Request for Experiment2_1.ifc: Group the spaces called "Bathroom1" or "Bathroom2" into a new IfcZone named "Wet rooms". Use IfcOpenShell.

First a look at what the model holds.

```python
import ifcopenshell

model = ifcopenshell.open("Experiment2_1.ifc")
print(model.schema)
seen = {}
for space in model.by_type("IfcSpace"):
    seen[space.LongName] = seen.get(space.LongName, 0) + 1
for name, count in sorted(seen.items(), key=str):
    print(count, "x", name)
print("zones:", [z.Name for z in model.by_type("IfcZone")][:20])
```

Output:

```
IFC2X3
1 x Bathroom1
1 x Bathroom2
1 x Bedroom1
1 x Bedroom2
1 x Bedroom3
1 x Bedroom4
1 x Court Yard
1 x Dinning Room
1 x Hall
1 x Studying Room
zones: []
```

```python
import ifcopenshell
import ifcopenshell.api.group
import ifcopenshell.api.root

model = ifcopenshell.open("Experiment2_1.ifc")

names = {"Bathroom1", "Bathroom2"}
spaces = [s for s in model.by_type("IfcSpace") if s.LongName in names]

zone = ifcopenshell.api.root.create_entity(model, ifc_class="IfcZone", name="Wet rooms")
ifcopenshell.api.group.assign_group(model, products=spaces, group=zone)
print(len(spaces), "spaces in", zone.Name)

model.write("Experiment2_1_rev.ifc")
```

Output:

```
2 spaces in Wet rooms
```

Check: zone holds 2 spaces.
